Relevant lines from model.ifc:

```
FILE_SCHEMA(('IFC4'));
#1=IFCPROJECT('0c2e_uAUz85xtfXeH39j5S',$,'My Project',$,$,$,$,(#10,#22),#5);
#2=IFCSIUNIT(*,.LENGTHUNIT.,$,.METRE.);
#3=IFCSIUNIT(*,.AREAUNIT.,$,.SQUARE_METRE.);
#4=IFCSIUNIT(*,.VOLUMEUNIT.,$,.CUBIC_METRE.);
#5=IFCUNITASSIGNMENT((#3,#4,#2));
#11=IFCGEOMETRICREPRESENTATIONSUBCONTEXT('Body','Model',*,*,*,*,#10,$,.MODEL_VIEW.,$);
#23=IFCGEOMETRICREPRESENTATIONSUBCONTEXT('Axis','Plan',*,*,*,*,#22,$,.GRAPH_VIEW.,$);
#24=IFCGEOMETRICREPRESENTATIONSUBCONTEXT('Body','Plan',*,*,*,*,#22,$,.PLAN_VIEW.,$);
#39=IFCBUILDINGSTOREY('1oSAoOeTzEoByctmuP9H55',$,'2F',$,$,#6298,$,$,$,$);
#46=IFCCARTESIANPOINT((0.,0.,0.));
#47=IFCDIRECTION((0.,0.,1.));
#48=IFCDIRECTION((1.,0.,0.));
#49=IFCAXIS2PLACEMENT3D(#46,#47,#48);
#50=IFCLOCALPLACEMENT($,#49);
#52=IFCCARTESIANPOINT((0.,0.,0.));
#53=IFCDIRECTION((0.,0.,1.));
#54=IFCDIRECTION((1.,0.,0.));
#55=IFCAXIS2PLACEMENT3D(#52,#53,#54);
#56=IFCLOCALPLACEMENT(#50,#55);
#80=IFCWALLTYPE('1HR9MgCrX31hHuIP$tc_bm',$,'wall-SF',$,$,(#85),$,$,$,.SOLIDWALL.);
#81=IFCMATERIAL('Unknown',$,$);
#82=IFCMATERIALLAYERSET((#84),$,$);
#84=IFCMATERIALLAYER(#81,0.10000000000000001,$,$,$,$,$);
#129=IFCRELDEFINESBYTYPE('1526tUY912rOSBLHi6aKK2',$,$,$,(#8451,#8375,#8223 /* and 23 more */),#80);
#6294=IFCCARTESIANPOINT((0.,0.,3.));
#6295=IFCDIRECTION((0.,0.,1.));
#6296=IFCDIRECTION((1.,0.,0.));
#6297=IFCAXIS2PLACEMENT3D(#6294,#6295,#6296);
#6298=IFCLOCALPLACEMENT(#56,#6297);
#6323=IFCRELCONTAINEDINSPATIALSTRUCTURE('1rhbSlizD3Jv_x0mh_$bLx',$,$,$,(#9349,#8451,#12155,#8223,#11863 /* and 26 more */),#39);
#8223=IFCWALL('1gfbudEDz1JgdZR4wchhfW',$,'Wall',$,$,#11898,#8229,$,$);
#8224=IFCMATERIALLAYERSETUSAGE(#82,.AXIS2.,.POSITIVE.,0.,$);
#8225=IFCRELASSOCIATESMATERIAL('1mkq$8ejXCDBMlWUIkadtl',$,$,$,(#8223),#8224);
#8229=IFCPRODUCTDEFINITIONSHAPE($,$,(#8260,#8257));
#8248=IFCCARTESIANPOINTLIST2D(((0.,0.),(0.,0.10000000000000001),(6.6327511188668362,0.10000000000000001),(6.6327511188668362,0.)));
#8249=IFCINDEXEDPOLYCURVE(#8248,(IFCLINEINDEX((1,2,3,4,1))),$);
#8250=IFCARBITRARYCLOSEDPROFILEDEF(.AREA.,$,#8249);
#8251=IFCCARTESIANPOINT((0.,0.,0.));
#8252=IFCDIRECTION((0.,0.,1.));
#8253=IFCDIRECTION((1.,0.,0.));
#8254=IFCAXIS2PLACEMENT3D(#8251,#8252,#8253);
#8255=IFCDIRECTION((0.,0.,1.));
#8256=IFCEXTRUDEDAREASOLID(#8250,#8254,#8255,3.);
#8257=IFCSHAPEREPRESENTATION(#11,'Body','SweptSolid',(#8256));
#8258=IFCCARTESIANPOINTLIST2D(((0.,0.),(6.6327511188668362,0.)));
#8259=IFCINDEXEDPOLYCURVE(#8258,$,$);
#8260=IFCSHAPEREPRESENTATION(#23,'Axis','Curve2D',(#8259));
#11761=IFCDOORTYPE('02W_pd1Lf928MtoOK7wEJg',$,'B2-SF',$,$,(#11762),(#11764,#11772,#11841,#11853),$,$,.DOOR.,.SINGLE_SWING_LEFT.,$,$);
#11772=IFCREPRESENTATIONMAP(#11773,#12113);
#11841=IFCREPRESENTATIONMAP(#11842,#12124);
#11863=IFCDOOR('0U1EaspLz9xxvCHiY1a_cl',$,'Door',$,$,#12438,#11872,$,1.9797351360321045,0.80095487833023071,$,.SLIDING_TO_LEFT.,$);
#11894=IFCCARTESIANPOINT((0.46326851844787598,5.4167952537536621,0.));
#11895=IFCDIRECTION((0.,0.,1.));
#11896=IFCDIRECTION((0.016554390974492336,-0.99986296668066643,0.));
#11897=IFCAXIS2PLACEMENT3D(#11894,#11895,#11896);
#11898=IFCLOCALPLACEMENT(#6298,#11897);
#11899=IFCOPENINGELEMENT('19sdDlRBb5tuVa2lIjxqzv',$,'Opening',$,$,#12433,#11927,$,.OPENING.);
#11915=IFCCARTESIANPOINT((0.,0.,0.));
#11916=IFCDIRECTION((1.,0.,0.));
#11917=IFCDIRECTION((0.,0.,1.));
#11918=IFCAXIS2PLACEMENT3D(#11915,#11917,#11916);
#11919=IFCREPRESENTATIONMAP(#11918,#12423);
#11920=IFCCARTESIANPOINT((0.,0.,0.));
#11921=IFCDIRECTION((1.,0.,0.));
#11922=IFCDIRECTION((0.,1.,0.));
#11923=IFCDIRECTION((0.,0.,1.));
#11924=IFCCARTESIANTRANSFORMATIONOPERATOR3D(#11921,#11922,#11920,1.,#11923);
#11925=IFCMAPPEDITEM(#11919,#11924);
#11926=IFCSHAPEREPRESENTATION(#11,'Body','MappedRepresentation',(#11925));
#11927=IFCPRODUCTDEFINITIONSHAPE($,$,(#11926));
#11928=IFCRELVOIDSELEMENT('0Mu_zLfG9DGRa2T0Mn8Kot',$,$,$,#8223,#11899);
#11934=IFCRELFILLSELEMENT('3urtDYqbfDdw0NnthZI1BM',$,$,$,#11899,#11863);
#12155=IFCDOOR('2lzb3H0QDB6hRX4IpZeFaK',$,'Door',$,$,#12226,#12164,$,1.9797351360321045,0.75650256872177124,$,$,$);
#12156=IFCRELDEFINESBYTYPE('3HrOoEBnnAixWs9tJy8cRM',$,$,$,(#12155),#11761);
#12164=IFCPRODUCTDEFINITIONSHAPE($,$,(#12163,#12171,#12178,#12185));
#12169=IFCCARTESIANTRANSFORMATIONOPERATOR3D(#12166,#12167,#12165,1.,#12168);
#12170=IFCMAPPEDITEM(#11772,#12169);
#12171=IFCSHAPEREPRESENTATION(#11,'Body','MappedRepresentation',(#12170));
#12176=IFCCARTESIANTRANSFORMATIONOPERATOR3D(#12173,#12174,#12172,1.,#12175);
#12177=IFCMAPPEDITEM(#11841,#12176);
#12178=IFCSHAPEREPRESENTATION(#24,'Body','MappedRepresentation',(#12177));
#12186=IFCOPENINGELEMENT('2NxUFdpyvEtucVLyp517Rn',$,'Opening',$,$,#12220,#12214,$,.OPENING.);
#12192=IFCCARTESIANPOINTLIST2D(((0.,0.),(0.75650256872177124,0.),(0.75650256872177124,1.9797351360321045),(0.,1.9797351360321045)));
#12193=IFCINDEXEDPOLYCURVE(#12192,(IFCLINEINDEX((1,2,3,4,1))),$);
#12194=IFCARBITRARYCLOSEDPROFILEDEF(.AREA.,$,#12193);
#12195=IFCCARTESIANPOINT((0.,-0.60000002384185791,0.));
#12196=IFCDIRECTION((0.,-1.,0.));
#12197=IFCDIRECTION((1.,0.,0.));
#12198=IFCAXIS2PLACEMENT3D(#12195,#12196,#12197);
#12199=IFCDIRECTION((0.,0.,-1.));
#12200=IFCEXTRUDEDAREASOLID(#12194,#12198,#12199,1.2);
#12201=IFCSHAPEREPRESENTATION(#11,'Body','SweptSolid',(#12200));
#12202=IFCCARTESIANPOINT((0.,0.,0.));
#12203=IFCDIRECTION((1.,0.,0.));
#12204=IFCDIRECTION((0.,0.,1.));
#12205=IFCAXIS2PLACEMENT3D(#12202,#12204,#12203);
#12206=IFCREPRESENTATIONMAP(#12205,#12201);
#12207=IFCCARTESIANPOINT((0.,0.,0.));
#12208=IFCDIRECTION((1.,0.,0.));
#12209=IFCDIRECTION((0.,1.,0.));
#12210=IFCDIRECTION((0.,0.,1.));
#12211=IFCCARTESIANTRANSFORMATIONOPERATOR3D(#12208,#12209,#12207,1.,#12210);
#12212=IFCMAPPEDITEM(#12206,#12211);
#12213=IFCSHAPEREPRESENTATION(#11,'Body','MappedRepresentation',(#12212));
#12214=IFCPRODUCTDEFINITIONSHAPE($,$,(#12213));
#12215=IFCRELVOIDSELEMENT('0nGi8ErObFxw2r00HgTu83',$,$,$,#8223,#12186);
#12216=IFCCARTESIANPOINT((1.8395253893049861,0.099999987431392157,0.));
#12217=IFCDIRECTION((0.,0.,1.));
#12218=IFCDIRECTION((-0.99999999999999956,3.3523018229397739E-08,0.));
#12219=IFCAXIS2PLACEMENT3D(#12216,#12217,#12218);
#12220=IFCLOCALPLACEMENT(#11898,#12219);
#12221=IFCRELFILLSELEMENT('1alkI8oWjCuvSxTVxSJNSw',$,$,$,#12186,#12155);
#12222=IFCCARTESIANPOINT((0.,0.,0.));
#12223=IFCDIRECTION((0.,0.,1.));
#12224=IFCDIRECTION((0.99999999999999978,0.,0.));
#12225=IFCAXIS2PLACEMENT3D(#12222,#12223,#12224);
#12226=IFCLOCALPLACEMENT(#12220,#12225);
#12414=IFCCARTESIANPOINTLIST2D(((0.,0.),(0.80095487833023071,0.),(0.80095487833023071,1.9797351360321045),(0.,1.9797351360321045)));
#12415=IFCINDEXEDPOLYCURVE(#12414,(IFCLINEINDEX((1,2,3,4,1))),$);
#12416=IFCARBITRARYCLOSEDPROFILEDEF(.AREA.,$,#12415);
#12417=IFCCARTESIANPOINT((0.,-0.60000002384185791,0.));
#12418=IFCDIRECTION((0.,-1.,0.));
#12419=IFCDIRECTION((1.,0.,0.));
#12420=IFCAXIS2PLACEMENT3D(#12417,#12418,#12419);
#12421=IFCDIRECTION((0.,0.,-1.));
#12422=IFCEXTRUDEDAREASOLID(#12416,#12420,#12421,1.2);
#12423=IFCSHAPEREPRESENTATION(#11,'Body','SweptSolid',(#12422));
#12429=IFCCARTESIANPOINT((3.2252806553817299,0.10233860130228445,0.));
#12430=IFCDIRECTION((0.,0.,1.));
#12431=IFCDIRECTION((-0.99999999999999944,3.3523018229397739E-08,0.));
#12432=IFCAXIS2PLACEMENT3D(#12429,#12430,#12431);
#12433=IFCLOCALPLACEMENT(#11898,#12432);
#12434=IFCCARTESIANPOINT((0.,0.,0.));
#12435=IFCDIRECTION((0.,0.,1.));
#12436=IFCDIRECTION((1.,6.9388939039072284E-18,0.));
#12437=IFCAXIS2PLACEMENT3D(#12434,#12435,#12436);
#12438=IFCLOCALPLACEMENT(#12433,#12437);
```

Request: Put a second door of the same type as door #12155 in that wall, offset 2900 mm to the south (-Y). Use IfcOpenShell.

```python
import ifcopenshell
import ifcopenshell.api.feature
import ifcopenshell.api.geometry
import ifcopenshell.api.root
import ifcopenshell.geom
import ifcopenshell.util.element
import ifcopenshell.util.placement
import ifcopenshell.util.shape

model = ifcopenshell.open("model.ifc")
settings = ifcopenshell.geom.settings()


def volume(element):
    """Net volume in cubic metres, openings subtracted."""
    shape = ifcopenshell.geom.create_shape(settings, element)
    return ifcopenshell.util.shape.get_volume(shape.geometry)


door = model.by_id(12155)
opening = door.FillsVoids[0].RelatingOpeningElement
wall = opening.VoidsElements[0].RelatingBuildingElement
before = volume(wall)
shift = ifcopenshell.util.placement.get_local_placement(wall.ObjectPlacement)[:3, 0] * 2.9

# copy_class copies the void relationship, type, container and properties, but no geometry.
new_opening = ifcopenshell.api.root.copy_class(model, product=opening)
new_opening.Representation = ifcopenshell.util.element.copy_deep(
    model, opening.Representation, exclude=["IfcGeometricRepresentationContext", "IfcRepresentationMap"]
)
new_door = ifcopenshell.api.root.copy_class(model, product=door)
new_door.Representation = ifcopenshell.util.element.copy_deep(
    model, door.Representation, exclude=["IfcGeometricRepresentationContext", "IfcRepresentationMap"]
)
ifcopenshell.api.feature.add_filling(model, opening=new_opening, element=new_door)

for old, new in ((opening, new_opening), (door, new_door)):
    matrix = ifcopenshell.util.placement.get_local_placement(old.ObjectPlacement)
    matrix[:3, 3] += shift
    ifcopenshell.api.geometry.edit_object_placement(model, product=new, matrix=matrix, is_si=False)

after = volume(wall)

print(f"wall volume {before:.3f} -> {after:.3f} m3")

model.write("model_rev.ifc")
```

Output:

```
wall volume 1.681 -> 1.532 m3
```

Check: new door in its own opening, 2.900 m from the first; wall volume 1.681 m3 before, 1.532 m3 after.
